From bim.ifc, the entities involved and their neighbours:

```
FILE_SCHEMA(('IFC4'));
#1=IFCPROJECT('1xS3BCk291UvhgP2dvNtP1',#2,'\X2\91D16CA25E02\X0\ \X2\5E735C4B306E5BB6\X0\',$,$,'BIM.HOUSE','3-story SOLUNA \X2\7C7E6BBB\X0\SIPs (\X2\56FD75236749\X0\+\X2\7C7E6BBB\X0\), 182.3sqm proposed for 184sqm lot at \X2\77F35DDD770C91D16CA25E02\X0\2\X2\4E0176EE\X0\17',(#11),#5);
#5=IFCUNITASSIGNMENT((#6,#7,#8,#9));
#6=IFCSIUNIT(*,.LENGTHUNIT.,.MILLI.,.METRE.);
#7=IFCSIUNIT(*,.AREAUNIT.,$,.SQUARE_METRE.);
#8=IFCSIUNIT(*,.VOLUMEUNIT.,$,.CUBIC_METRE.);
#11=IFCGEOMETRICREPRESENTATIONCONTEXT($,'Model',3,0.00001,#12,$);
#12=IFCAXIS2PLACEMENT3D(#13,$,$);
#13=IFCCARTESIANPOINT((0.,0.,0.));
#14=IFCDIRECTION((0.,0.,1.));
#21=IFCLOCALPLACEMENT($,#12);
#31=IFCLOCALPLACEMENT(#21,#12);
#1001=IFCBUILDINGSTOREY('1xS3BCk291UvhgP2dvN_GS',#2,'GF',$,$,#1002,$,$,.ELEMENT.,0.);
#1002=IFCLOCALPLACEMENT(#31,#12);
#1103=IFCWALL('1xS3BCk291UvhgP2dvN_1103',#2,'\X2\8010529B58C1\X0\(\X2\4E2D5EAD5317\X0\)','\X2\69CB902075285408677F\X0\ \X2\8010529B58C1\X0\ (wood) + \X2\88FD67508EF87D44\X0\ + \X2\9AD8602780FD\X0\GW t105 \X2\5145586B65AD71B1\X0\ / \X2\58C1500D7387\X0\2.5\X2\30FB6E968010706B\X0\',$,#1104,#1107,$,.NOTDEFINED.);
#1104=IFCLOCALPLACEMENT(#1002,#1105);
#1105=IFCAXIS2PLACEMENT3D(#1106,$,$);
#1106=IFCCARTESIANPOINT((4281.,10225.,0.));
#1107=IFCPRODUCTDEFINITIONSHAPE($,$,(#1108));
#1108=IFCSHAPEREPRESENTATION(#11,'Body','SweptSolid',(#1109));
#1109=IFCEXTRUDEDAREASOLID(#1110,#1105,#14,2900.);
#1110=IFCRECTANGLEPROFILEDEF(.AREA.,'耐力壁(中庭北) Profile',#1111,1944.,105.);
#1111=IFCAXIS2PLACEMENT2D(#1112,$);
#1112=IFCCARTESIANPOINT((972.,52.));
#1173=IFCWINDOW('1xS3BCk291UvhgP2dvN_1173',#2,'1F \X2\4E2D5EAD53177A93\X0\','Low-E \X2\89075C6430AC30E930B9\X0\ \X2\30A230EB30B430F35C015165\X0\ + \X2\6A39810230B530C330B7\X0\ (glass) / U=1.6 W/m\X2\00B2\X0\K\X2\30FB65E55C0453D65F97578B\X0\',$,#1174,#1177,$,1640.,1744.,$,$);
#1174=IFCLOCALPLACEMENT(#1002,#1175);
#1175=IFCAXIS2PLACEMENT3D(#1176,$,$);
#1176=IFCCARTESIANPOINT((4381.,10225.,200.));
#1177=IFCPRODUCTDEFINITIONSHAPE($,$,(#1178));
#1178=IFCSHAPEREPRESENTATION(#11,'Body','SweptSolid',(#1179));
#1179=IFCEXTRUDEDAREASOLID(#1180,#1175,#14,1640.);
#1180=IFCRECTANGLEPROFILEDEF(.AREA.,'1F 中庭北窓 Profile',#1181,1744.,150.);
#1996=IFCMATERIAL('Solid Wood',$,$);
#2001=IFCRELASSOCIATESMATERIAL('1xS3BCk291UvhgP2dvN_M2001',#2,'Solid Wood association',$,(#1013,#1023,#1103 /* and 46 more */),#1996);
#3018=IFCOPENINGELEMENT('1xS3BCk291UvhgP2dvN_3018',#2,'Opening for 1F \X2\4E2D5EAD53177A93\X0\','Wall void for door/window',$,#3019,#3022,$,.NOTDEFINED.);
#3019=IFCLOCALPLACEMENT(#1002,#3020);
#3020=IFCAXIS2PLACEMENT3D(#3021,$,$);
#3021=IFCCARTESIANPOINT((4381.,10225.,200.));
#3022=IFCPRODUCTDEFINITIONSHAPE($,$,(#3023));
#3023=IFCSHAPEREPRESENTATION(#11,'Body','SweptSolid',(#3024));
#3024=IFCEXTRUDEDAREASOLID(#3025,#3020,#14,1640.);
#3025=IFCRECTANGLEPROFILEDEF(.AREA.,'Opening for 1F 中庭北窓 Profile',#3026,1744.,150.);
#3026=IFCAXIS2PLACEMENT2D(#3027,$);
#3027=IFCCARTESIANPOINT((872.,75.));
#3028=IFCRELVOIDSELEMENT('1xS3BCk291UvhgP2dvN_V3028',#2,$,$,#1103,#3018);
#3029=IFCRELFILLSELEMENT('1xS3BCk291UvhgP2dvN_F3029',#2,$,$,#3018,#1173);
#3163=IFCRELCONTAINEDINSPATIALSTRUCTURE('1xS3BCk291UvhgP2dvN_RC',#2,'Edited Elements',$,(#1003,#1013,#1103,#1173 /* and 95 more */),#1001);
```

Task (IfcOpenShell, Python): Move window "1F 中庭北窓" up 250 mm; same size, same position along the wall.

```python
import numpy as np
import ifcopenshell
import ifcopenshell.api.geometry
import ifcopenshell.util.placement
import ifcopenshell.util.unit

model = ifcopenshell.open("bim.ifc")
unit_scale = ifcopenshell.util.unit.calculate_unit_scale(model)

window = model.by_id(1173)
opening = window.FillsVoids[0].RelatingOpeningElement
dz = 0.25 / unit_scale

shift = np.array([0.0, 0.0, dz])
# The window is not placed relative to its opening, so move both.
for product in (opening, window):
    matrix = ifcopenshell.util.placement.get_local_placement(product.ObjectPlacement)
    matrix[:3, 3] += shift
    ifcopenshell.api.geometry.edit_object_placement(model, product=product, matrix=matrix, is_si=False)

print(f"moved by {dz * unit_scale:+.3f} m")

model.write("bim-out.ifc")
```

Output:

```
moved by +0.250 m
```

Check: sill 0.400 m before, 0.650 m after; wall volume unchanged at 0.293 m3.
